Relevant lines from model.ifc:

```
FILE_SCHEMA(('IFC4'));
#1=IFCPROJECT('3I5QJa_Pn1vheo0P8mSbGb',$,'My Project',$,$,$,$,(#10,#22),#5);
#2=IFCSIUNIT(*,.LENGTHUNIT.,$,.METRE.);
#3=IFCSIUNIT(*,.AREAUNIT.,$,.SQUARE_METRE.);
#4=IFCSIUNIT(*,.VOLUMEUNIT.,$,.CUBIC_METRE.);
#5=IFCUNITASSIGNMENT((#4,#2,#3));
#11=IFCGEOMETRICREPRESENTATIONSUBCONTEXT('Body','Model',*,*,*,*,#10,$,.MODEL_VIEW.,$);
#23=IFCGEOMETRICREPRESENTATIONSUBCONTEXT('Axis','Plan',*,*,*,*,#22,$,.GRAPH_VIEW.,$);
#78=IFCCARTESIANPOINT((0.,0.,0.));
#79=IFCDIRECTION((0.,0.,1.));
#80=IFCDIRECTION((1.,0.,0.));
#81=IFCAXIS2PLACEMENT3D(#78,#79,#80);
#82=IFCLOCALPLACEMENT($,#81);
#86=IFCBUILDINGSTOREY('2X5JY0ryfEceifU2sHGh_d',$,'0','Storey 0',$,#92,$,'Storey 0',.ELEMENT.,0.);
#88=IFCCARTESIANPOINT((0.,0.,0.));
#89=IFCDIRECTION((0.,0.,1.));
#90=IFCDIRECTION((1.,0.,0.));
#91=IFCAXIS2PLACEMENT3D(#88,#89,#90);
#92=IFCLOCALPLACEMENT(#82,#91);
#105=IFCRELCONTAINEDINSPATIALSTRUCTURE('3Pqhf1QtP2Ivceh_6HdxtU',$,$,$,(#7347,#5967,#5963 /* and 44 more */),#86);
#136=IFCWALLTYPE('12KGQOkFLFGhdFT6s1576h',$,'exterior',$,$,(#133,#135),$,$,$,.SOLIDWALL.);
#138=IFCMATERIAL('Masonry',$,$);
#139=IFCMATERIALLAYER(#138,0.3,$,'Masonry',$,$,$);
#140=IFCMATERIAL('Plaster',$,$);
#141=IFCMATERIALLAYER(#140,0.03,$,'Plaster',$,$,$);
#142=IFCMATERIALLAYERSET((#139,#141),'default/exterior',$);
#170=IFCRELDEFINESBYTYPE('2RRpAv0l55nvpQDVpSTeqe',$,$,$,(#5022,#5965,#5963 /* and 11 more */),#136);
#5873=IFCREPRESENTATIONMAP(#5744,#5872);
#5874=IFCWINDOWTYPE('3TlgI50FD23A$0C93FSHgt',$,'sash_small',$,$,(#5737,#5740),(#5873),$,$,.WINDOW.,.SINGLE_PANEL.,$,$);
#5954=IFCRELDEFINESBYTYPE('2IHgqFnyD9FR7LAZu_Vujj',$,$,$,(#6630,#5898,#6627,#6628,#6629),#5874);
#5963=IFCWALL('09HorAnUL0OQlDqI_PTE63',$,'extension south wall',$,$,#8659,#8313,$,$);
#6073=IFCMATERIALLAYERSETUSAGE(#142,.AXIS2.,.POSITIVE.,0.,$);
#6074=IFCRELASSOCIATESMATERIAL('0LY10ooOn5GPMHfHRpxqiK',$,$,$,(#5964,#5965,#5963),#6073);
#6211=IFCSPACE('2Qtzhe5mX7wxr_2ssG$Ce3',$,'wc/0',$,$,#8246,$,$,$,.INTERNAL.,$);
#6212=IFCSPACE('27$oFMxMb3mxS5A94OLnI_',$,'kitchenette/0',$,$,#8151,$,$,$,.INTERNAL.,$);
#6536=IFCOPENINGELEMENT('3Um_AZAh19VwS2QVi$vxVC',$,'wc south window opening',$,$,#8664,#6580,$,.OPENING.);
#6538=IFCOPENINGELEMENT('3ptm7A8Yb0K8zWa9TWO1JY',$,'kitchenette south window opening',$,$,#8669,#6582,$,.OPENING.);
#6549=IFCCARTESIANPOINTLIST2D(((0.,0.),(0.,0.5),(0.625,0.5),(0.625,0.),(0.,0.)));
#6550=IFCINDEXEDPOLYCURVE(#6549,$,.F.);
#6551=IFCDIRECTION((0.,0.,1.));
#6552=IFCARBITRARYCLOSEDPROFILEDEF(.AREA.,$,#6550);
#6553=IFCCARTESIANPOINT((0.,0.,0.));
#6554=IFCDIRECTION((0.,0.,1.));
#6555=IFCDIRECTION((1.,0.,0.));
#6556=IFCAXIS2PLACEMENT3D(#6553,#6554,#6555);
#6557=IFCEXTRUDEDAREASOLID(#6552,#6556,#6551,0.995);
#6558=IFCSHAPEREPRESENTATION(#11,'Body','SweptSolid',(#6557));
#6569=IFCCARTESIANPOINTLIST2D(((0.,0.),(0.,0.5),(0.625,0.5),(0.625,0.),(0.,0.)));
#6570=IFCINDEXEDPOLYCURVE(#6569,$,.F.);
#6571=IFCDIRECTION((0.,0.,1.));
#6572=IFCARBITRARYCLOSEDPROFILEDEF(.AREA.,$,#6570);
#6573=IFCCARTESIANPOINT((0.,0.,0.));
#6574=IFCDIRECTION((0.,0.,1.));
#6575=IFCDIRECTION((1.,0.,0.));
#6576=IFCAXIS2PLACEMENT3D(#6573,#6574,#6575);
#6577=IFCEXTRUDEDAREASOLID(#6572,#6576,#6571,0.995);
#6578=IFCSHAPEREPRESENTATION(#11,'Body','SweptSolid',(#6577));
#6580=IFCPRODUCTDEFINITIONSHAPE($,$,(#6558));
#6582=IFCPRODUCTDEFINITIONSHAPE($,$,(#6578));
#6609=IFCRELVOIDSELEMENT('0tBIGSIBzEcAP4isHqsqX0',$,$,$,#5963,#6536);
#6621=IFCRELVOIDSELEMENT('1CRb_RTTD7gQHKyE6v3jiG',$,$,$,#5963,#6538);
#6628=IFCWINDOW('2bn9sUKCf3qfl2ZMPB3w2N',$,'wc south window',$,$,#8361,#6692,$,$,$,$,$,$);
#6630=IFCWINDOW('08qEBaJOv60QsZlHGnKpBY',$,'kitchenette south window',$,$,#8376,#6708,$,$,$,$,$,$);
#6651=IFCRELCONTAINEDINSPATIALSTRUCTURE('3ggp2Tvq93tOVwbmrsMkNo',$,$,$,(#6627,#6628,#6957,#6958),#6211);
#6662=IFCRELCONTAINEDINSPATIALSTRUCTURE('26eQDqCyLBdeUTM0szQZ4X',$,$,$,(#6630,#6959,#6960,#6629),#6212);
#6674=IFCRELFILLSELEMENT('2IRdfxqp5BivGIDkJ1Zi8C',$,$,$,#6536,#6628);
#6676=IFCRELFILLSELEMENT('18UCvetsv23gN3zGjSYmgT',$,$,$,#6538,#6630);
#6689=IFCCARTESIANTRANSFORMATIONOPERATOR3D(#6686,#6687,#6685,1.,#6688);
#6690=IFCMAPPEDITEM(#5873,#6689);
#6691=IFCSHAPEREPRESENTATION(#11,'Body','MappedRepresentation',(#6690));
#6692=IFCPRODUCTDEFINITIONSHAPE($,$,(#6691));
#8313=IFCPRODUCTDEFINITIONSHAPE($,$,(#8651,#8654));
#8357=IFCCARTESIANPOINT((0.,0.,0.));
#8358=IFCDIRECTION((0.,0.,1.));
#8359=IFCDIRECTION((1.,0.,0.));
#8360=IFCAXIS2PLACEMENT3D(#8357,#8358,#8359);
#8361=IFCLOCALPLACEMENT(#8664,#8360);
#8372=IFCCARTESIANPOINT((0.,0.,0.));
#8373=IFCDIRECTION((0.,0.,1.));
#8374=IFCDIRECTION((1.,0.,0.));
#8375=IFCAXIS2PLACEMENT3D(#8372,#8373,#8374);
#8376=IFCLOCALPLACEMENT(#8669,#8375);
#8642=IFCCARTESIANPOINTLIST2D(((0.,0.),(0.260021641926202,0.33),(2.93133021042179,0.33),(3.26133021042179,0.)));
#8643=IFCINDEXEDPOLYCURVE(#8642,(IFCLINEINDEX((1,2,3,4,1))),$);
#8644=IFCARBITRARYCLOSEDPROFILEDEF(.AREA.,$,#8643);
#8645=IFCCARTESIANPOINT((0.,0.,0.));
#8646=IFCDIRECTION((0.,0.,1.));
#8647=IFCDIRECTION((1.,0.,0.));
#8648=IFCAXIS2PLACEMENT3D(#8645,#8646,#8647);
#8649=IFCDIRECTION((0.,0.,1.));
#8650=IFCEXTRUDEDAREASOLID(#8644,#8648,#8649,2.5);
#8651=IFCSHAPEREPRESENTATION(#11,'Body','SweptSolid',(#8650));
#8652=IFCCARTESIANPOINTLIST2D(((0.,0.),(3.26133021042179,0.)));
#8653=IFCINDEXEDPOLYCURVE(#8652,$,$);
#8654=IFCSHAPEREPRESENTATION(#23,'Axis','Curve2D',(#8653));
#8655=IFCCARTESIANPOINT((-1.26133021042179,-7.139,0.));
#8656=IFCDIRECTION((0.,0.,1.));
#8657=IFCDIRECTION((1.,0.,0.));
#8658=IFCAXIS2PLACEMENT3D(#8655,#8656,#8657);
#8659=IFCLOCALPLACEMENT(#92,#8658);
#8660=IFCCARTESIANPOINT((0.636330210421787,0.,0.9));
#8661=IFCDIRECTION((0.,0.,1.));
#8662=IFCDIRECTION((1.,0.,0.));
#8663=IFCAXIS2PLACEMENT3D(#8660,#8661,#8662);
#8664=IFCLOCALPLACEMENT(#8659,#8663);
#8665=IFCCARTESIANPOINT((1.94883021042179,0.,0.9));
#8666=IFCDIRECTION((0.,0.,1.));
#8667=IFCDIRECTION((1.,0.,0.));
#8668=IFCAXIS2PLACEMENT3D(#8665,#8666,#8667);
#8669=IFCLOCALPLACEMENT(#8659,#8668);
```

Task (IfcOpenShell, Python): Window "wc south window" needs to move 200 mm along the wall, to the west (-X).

```python
import ifcopenshell
import ifcopenshell.api.geometry
import ifcopenshell.util.placement
import ifcopenshell.util.unit

model = ifcopenshell.open("model.ifc")
unit_scale = ifcopenshell.util.unit.calculate_unit_scale(model)

window = model.by_guid("2bn9sUKCf3qfl2ZMPB3w2N")
opening = window.FillsVoids[0].RelatingOpeningElement
wall = opening.VoidsElements[0].RelatingBuildingElement

wall_matrix = ifcopenshell.util.placement.get_local_placement(wall.ObjectPlacement)
shift = wall_matrix[:3, 0] * -0.2 / unit_scale
before = ifcopenshell.util.placement.get_local_placement(window.ObjectPlacement)[:3, 3].copy()

# The window is placed relative to its opening, so it follows when the opening moves.
matrix = ifcopenshell.util.placement.get_local_placement(opening.ObjectPlacement)
matrix[:3, 3] += shift
ifcopenshell.api.geometry.edit_object_placement(
    model, product=opening, matrix=matrix, is_si=False, should_transform_children=True
)

after = ifcopenshell.util.placement.get_local_placement(window.ObjectPlacement)[:3, 3]
print("window moved by", (after - before).round(3) + 0.0)

model.write("model-out.ifc")
```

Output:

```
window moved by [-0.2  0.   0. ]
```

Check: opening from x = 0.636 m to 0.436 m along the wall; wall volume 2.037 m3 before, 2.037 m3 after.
